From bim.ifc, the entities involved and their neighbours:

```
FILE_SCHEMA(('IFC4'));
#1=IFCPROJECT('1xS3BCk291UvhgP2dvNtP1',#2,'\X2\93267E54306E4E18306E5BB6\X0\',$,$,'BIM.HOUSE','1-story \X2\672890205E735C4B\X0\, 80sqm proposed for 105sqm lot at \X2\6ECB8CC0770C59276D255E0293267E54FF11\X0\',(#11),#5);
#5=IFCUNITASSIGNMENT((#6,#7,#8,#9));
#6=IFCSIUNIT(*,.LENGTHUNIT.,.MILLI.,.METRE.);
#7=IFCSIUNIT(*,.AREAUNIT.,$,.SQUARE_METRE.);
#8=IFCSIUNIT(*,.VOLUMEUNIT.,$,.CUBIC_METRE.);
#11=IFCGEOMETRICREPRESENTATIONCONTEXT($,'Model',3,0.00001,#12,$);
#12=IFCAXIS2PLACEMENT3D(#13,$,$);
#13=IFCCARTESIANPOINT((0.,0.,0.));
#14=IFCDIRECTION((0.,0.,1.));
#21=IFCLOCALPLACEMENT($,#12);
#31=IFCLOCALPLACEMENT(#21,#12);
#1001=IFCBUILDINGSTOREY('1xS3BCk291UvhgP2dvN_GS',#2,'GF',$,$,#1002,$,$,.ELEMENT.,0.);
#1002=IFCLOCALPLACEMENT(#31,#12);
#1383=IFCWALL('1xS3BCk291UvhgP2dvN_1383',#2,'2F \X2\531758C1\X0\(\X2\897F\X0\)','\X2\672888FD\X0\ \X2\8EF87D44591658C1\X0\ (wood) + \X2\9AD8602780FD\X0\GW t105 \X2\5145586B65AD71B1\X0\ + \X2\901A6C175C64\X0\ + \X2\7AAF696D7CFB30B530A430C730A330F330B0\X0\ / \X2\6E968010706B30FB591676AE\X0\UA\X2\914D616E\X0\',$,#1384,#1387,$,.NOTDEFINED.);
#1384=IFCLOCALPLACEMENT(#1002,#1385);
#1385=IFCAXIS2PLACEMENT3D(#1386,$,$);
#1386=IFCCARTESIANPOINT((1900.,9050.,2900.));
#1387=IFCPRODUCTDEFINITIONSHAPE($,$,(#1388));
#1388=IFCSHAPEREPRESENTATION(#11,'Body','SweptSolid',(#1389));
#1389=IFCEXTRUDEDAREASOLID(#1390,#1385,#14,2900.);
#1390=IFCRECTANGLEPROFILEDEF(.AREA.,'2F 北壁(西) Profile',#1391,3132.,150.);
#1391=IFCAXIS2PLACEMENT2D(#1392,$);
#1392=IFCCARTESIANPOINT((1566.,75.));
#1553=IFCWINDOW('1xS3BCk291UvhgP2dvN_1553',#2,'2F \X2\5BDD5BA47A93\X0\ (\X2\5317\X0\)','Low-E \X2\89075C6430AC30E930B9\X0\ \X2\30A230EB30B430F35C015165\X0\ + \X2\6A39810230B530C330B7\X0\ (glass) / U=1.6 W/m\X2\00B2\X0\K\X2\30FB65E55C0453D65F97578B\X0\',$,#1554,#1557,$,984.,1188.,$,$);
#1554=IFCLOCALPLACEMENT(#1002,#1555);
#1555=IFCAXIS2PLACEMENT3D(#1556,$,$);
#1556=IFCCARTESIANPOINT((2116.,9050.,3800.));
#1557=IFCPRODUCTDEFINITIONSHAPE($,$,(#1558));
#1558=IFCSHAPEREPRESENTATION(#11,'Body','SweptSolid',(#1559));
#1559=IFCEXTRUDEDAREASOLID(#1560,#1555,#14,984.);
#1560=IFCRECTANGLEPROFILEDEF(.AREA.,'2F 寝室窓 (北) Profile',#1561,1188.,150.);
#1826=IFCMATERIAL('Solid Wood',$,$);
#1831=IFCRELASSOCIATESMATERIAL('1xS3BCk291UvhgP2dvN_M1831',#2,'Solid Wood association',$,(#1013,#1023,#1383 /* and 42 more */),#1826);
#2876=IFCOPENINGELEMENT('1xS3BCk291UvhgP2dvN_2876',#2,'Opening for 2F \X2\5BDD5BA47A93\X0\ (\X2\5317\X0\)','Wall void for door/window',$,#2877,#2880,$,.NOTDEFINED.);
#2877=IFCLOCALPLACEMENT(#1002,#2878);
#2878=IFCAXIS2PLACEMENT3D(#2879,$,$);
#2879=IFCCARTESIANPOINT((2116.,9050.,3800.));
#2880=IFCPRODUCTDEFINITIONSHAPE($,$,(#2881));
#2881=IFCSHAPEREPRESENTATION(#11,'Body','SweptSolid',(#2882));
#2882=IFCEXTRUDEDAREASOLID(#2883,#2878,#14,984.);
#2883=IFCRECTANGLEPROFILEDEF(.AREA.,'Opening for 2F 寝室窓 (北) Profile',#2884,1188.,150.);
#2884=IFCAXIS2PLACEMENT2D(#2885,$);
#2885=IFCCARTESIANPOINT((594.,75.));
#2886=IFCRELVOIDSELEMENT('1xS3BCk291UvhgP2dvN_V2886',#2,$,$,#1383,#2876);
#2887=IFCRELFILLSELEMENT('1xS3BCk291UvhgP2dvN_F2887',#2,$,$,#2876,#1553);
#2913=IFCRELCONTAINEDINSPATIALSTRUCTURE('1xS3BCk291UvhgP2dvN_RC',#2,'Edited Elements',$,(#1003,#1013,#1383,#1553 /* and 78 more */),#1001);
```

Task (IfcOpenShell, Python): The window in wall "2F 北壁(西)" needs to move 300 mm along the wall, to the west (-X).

```python
import ifcopenshell
import ifcopenshell.api.geometry
import ifcopenshell.util.placement

model = ifcopenshell.open("bim.ifc")

window = model.by_guid("1xS3BCk291UvhgP2dvN_1553")
opening = window.FillsVoids[0].RelatingOpeningElement
wall = opening.VoidsElements[0].RelatingBuildingElement

wall_matrix = ifcopenshell.util.placement.get_local_placement(wall.ObjectPlacement)
shift = wall_matrix[:3, 0] * -300.0
before = ifcopenshell.util.placement.get_local_placement(window.ObjectPlacement)[:3, 3].copy()

# The window is not placed relative to its opening, so move both.
for product in (opening, window):
    matrix = ifcopenshell.util.placement.get_local_placement(product.ObjectPlacement)
    matrix[:3, 3] += shift
    ifcopenshell.api.geometry.edit_object_placement(model, product=product, matrix=matrix, is_si=False)

after = ifcopenshell.util.placement.get_local_placement(window.ObjectPlacement)[:3, 3]
print("window moved by", (after - before).round(3) + 0.0)

model.write("bim_v2.ifc")
```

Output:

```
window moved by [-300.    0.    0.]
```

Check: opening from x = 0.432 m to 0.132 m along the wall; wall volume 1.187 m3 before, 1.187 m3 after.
